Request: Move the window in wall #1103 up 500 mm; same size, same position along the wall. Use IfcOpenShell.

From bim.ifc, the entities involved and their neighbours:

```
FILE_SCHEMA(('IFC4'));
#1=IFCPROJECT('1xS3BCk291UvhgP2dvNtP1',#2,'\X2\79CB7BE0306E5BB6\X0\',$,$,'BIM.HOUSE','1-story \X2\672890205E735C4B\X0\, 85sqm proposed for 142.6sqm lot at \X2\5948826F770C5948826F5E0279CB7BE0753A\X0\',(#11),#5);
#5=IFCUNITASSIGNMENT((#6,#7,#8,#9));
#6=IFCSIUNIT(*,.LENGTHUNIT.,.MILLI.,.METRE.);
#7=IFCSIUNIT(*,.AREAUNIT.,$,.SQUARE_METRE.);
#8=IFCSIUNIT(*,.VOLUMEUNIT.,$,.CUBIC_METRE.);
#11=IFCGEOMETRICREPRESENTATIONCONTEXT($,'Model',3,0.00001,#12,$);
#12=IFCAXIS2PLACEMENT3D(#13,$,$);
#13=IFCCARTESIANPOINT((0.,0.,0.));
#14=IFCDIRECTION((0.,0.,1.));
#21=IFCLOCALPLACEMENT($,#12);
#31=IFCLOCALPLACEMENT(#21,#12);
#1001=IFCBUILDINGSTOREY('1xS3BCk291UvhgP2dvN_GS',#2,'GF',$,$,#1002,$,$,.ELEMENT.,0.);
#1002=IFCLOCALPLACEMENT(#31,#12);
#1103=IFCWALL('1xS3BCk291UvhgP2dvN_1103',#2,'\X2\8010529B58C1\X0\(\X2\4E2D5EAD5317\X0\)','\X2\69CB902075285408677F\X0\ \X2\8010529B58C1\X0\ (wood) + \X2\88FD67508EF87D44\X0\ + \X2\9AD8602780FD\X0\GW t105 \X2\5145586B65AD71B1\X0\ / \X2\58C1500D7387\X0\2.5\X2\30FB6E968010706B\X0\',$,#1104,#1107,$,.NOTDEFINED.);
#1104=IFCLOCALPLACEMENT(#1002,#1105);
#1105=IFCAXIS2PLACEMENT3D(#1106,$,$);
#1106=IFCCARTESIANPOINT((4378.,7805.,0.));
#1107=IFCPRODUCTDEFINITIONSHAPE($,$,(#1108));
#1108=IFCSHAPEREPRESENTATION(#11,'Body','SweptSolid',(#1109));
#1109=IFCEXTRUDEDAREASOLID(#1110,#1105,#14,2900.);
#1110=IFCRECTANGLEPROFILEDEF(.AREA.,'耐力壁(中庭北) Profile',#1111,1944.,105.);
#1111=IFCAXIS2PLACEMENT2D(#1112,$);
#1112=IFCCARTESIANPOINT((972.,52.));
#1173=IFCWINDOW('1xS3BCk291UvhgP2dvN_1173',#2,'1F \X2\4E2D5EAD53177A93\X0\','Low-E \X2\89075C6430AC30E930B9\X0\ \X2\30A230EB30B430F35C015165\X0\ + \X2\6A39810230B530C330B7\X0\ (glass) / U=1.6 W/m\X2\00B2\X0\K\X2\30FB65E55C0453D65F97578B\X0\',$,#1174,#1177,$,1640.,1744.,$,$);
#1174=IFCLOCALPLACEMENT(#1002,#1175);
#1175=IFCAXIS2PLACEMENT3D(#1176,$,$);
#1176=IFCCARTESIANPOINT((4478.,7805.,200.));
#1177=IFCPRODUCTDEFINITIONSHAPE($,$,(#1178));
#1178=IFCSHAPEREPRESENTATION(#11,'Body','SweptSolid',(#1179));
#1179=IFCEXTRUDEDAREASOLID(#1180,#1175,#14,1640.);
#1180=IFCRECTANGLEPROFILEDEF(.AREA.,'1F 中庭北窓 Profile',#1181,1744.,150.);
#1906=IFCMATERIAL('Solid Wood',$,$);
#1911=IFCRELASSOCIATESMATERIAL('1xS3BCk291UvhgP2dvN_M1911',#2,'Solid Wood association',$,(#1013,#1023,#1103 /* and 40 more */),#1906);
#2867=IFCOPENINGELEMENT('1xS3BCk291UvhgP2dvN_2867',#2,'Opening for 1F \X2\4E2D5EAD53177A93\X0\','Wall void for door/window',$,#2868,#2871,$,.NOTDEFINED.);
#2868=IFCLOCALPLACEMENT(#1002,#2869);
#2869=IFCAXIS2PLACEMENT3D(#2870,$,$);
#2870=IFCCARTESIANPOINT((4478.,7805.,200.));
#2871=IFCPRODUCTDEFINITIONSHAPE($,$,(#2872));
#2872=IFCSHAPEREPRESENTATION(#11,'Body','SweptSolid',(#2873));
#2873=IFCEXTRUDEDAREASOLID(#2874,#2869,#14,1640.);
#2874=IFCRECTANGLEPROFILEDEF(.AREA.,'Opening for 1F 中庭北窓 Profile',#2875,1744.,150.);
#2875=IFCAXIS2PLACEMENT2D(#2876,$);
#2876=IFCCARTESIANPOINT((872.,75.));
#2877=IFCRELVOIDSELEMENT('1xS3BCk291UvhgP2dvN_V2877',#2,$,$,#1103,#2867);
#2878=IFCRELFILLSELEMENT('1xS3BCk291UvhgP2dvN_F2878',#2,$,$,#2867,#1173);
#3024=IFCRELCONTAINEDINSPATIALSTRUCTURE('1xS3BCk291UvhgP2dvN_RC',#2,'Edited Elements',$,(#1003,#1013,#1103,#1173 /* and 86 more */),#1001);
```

```python
import numpy as np
import ifcopenshell
import ifcopenshell.api.geometry
import ifcopenshell.util.placement
import ifcopenshell.util.unit

model = ifcopenshell.open("bim.ifc")
unit_scale = ifcopenshell.util.unit.calculate_unit_scale(model)

window = model.by_guid("1xS3BCk291UvhgP2dvN_1173")
opening = window.FillsVoids[0].RelatingOpeningElement
dz = 0.5 / unit_scale

shift = np.array([0.0, 0.0, dz])
# The window is not placed relative to its opening, so move both.
for product in (opening, window):
    matrix = ifcopenshell.util.placement.get_local_placement(product.ObjectPlacement)
    matrix[:3, 3] += shift
    ifcopenshell.api.geometry.edit_object_placement(model, product=product, matrix=matrix, is_si=False)

print(f"moved by {dz * unit_scale:+.3f} m")

model.write("bim_v2.ifc")
```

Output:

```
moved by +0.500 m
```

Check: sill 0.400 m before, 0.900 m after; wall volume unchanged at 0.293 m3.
